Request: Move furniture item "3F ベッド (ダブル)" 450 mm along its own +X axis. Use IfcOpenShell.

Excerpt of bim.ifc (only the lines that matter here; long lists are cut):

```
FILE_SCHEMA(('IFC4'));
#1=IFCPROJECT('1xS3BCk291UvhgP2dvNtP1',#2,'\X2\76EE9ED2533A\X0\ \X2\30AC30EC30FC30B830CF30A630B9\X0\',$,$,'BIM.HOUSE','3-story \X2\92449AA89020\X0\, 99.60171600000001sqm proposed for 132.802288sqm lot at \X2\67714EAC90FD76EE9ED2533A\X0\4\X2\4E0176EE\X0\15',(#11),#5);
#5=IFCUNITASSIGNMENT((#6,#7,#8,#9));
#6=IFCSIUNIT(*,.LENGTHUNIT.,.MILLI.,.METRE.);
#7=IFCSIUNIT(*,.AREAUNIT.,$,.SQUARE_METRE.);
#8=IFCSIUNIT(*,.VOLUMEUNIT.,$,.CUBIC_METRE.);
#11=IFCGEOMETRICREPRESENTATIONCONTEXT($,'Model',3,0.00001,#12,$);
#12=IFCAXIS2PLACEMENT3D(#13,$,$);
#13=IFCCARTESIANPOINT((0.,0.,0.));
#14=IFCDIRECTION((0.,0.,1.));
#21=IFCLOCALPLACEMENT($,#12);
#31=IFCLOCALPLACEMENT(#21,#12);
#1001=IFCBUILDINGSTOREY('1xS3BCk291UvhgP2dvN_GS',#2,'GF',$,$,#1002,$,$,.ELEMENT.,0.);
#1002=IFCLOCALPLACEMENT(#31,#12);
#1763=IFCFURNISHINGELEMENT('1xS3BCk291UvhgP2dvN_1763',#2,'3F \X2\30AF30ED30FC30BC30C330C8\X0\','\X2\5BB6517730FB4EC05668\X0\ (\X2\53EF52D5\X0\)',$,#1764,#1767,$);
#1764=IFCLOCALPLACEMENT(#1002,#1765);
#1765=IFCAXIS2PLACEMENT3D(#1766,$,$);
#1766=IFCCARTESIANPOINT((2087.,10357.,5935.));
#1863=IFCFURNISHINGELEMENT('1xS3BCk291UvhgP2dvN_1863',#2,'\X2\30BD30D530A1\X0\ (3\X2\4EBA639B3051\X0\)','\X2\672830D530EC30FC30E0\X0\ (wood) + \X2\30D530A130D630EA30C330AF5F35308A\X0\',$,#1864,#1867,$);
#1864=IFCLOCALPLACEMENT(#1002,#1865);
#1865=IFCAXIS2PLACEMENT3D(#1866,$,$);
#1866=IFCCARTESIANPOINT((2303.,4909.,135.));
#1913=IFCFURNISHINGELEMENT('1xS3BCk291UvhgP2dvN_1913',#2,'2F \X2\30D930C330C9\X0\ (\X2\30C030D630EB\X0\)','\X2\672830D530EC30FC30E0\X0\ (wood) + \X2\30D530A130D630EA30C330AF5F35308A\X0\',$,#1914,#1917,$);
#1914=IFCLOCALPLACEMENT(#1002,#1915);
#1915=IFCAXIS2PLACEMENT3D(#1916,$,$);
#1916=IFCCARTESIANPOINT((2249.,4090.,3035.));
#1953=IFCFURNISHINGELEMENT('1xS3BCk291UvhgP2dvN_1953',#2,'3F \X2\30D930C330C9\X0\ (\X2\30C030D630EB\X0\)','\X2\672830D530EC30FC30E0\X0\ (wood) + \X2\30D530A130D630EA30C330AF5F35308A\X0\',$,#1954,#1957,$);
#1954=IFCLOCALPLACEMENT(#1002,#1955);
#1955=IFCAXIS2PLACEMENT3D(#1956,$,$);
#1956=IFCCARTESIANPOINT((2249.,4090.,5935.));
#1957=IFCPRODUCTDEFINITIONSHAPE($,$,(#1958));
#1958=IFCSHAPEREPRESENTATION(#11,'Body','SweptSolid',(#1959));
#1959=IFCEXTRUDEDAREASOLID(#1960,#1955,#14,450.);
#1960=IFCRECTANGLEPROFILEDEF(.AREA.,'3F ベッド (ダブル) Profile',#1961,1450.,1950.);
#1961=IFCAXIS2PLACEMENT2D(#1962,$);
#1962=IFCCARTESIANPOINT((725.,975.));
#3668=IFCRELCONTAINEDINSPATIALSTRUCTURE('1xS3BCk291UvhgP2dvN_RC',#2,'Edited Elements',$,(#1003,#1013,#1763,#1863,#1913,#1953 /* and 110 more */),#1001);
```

```python
import ifcopenshell
import ifcopenshell.api.geometry
import ifcopenshell.util.placement
import ifcopenshell.util.unit

model = ifcopenshell.open("bim.ifc")
unit_scale = ifcopenshell.util.unit.calculate_unit_scale(model)

item = model.by_guid("1xS3BCk291UvhgP2dvN_1953")
matrix = ifcopenshell.util.placement.get_local_placement(item.ObjectPlacement)
matrix[:3, 3] += matrix[:3, 0] * 0.45 / unit_scale
ifcopenshell.api.geometry.edit_object_placement(model, product=item, matrix=matrix, is_si=False)

print(ifcopenshell.util.placement.get_local_placement(item.ObjectPlacement).round(3) + 0.0)

model.write("bim_v2.ifc")
```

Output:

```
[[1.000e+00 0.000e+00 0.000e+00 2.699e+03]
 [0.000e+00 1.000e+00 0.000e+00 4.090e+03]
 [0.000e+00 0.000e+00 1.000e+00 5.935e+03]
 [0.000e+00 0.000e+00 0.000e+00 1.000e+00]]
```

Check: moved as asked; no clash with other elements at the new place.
